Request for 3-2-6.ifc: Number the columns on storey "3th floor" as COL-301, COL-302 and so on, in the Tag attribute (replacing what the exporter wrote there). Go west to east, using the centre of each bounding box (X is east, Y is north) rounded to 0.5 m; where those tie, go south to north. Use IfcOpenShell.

First a look at what the model holds.

```python
import ifcopenshell
import ifcopenshell.util.element
import ifcopenshell.util.placement

model = ifcopenshell.open("3-2-6.ifc")
print(model.schema)
storey = next(s for s in model.by_type("IfcBuildingStorey") if s.Name == "3th floor")
columns = [e for e in ifcopenshell.util.element.get_decomposition(storey) if e.is_a("IfcColumn")]
for e in sorted(columns, key=lambda e: e.id()):
    origin = ifcopenshell.util.placement.get_local_placement(e.ObjectPlacement)[:3, 3]
    print(e.id(), e.Tag, e.Name, origin.round(2) + 0.0, sep=" | ")
```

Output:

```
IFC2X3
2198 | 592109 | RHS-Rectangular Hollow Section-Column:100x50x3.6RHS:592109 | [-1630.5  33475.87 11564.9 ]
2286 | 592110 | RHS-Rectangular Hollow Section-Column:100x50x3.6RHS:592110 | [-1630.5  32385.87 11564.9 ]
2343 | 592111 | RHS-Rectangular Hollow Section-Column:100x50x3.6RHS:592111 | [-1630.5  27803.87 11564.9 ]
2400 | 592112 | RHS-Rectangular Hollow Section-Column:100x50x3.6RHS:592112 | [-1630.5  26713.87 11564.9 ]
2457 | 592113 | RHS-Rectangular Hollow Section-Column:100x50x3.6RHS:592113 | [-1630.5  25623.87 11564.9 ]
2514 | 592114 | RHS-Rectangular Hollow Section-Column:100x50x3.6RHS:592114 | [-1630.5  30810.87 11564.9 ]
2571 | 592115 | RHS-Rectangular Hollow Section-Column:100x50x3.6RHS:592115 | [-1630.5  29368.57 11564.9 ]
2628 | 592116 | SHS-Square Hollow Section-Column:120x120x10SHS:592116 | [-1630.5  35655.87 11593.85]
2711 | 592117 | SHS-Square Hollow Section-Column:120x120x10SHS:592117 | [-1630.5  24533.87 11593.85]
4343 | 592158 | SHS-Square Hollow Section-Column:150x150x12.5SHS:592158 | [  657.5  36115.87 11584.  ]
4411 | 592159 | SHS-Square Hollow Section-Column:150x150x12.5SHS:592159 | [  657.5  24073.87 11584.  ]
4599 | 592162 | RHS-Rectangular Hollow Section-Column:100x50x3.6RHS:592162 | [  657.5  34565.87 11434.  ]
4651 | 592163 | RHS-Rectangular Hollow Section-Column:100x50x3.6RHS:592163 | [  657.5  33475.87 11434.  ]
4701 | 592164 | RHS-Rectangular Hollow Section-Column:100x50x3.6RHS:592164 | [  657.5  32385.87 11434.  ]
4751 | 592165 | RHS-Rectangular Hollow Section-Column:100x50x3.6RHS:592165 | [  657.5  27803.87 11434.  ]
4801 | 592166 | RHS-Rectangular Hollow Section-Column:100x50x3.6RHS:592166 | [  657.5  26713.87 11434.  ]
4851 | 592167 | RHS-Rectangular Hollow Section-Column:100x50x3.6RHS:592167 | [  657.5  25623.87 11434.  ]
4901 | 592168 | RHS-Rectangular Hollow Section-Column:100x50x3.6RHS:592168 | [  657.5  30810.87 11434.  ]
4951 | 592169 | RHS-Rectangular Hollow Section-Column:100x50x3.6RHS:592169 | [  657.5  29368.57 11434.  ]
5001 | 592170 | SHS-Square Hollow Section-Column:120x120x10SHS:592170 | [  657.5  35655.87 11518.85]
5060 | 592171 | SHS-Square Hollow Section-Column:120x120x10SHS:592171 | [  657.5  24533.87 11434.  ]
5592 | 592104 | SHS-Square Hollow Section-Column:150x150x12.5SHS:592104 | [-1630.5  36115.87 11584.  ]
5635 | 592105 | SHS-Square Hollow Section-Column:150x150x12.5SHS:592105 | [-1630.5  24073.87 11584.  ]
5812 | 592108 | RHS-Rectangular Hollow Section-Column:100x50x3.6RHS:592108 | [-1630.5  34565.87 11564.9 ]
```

```python
import ifcopenshell
import ifcopenshell.geom
import ifcopenshell.util.element
import ifcopenshell.util.shape

model = ifcopenshell.open("3-2-6.ifc")
settings = ifcopenshell.geom.settings()
settings.set("use-world-coords", True)


def centre(element):
    shape = ifcopenshell.geom.create_shape(settings, element)
    return ifcopenshell.util.shape.get_bbox_centroid(shape.geometry)


storey = next(s for s in model.by_type("IfcBuildingStorey") if s.Name == "3th floor")
columns = [e for e in ifcopenshell.util.element.get_decomposition(storey) if e.is_a("IfcColumn")]

# Insertion points can sit at a corner or the storey origin, so sort by the geometry (in metres).
centres = {e: centre(e) for e in columns}
columns.sort(key=lambda e: (round(centres[e][0] / 0.5), centres[e][1]))

for i, e in enumerate(columns, start=1):
    number = f"COL-3{i:02d}"
    e.Tag = number
    print(e.id(), number)

model.write("3-2-6_updated.ifc")
```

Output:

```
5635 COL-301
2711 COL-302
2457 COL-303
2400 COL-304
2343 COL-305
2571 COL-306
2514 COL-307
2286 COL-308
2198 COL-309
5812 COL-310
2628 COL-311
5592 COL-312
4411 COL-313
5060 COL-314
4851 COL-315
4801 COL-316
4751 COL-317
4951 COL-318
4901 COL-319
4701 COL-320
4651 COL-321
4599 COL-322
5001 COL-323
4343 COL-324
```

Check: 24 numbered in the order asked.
